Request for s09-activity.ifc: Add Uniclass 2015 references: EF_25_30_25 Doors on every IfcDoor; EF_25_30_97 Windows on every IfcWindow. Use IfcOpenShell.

First a look at what the model holds.

```python
import ifcopenshell

model = ifcopenshell.open("s09-activity.ifc")
print(model.schema)
print("classifications:", [c.Name for c in model.by_type("IfcClassification")])
for ifc_class in ("IfcDoor", "IfcRoof", "IfcStair", "IfcWall", "IfcWindow"):
    print(ifc_class, len(model.by_type(ifc_class)))
```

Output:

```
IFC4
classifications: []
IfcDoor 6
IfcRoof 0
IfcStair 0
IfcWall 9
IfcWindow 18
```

```python
import ifcopenshell
import ifcopenshell.api.classification

model = ifcopenshell.open("s09-activity.ifc")

system = ifcopenshell.api.classification.add_classification(model, classification="Uniclass 2015")

codes = {
    "IfcDoor": ("EF_25_30_25", "Doors"),
    "IfcWindow": ("EF_25_30_97", "Windows"),
}
for ifc_class, (code, name) in codes.items():
    products = model.by_type(ifc_class)
    ifcopenshell.api.classification.add_reference(
        model, products=products, classification=system, identification=code, name=name
    )
    print(code, len(products))

model.write("s09-activity-out.ifc")
```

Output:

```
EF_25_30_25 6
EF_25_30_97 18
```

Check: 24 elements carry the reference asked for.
